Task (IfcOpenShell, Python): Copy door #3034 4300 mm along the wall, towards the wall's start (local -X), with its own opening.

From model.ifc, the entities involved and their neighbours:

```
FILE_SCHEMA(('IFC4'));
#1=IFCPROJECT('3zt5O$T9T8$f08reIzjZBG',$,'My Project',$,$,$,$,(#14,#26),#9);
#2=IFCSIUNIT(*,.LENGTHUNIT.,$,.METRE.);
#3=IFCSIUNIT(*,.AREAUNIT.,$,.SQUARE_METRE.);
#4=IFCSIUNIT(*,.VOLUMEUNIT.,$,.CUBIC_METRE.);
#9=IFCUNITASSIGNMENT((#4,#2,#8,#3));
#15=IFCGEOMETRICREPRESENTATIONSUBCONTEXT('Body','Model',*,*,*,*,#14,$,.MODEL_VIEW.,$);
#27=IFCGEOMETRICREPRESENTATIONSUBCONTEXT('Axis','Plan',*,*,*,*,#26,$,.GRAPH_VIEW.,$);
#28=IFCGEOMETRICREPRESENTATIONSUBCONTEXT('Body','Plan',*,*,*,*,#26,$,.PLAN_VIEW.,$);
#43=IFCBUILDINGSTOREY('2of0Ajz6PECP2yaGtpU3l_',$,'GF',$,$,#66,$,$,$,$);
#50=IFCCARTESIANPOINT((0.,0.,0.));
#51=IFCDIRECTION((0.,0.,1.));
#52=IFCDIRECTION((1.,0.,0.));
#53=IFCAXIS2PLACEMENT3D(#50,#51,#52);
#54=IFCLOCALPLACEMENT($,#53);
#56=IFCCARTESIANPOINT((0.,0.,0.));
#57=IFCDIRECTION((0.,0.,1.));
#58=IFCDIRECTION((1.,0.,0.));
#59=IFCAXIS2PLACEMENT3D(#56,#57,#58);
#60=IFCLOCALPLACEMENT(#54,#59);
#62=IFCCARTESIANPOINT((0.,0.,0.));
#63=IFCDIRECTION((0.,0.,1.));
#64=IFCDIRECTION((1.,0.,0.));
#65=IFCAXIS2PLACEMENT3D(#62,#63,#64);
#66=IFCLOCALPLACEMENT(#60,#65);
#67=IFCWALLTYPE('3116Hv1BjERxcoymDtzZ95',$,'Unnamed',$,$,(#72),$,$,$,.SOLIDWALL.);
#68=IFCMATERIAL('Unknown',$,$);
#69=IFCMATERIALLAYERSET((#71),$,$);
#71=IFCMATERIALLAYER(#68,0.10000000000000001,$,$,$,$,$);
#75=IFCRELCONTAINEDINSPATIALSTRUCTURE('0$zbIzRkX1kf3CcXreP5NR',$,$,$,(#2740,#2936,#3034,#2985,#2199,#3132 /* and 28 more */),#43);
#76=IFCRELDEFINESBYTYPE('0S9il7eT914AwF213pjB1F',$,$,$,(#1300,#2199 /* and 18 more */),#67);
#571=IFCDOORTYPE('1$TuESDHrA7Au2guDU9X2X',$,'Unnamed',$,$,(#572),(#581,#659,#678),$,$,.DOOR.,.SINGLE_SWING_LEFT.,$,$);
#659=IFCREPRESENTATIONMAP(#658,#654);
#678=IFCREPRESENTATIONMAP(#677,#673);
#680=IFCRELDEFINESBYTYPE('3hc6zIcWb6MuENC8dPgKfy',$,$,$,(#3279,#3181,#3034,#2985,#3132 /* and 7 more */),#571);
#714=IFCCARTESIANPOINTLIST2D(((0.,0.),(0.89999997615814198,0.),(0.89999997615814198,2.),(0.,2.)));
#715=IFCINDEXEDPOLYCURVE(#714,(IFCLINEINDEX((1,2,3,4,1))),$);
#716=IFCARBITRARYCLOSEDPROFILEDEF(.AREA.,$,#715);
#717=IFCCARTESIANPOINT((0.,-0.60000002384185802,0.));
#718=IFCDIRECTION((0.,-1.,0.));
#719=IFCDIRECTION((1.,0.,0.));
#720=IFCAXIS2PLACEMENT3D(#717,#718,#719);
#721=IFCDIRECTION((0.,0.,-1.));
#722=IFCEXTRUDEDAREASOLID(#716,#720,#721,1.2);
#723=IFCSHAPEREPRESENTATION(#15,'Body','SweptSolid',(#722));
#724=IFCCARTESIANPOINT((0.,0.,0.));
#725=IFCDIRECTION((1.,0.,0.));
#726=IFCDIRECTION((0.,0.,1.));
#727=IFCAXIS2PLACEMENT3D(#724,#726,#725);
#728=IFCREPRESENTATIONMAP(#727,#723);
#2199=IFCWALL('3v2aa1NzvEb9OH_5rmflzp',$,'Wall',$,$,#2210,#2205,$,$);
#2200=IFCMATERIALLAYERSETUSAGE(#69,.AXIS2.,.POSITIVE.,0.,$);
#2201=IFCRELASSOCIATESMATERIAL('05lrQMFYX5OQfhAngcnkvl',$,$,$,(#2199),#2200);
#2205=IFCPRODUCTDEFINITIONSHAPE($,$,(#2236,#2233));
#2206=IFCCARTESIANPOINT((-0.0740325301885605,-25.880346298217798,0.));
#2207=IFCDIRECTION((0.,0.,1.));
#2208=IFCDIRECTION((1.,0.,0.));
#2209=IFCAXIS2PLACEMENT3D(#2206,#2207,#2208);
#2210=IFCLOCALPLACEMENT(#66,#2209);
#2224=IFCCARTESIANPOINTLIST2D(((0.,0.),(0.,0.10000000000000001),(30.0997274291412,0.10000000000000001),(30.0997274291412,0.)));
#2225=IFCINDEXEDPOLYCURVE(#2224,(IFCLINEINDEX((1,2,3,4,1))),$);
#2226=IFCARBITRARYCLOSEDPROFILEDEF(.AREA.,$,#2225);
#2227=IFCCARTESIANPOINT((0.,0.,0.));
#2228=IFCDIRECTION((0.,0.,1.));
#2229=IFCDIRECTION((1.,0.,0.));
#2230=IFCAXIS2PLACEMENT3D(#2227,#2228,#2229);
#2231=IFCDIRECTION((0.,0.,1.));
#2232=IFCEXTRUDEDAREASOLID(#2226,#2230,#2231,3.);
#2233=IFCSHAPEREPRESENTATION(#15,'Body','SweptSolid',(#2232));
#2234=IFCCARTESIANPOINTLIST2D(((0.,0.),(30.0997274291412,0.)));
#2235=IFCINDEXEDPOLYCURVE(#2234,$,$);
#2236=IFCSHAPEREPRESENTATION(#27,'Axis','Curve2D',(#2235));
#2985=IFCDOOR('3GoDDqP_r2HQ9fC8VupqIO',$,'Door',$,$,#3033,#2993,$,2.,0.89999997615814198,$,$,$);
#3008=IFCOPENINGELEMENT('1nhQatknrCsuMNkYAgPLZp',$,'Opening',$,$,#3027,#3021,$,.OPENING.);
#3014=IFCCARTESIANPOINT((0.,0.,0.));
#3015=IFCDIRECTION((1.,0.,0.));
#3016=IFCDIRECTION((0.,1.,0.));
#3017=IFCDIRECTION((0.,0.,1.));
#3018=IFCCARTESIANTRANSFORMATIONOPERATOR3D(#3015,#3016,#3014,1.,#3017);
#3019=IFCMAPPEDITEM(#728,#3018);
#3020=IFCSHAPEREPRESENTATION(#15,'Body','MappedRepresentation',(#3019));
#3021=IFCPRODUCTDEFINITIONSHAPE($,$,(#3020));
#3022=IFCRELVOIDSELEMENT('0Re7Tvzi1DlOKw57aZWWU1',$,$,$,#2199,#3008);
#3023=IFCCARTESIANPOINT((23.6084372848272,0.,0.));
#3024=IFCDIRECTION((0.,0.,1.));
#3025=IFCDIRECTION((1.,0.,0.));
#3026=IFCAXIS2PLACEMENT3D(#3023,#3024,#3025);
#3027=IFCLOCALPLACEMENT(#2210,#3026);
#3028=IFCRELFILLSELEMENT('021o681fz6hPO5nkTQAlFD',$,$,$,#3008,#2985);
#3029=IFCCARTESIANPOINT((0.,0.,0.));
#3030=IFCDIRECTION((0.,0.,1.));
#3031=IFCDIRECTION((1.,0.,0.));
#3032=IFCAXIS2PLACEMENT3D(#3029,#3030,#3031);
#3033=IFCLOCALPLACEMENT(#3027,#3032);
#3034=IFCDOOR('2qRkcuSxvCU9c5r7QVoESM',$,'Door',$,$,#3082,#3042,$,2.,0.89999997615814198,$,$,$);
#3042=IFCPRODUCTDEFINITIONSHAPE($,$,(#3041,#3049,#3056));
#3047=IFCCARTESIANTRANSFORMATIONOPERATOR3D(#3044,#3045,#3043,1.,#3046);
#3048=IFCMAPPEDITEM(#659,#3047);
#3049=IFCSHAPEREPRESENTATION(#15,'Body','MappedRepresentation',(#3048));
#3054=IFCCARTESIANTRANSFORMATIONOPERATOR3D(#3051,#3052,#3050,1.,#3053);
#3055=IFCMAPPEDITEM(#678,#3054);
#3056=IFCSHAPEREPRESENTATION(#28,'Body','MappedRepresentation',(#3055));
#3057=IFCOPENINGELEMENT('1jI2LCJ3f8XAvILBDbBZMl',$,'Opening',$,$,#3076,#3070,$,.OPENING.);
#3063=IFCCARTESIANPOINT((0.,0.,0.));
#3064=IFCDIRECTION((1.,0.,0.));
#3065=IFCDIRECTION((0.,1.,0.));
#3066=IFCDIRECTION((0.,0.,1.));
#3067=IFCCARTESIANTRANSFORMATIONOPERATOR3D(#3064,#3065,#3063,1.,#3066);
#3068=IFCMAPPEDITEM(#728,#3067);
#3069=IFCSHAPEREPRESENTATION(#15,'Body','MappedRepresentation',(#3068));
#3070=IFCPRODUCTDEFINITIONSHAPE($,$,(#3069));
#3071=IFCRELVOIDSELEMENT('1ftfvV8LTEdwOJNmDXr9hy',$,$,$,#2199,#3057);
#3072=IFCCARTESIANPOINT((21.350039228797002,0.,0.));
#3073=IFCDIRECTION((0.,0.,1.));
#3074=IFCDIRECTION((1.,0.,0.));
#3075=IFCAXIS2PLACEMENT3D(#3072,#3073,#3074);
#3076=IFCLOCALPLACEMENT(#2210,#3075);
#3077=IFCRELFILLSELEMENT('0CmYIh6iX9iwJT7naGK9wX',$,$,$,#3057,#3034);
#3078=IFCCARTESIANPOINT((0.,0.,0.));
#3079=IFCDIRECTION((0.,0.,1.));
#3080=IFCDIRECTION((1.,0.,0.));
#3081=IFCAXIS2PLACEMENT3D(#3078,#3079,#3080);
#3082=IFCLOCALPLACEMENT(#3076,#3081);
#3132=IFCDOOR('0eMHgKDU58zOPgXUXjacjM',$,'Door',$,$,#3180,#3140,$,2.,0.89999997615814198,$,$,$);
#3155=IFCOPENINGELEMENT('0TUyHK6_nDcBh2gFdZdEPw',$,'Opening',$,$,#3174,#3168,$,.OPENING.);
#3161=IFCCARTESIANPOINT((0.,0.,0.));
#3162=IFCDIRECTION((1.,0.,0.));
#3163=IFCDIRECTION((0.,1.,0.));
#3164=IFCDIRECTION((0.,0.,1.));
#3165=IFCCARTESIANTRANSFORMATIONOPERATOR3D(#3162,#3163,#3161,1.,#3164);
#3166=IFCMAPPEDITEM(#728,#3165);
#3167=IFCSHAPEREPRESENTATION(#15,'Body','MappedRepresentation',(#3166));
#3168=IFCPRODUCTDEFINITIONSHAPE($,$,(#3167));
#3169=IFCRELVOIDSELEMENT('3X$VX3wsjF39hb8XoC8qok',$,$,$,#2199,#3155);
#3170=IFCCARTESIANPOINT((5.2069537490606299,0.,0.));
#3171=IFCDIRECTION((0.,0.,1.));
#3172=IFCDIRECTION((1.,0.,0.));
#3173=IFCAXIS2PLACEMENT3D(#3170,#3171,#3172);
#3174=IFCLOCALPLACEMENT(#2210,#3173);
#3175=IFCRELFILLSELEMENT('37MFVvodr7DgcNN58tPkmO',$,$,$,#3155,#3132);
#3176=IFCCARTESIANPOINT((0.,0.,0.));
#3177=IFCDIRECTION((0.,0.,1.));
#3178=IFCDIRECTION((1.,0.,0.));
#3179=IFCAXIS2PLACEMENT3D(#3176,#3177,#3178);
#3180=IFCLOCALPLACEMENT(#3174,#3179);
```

```python
import ifcopenshell
import ifcopenshell.api.feature
import ifcopenshell.api.geometry
import ifcopenshell.api.root
import ifcopenshell.geom
import ifcopenshell.util.element
import ifcopenshell.util.placement
import ifcopenshell.util.shape

model = ifcopenshell.open("model.ifc")
settings = ifcopenshell.geom.settings()


def volume(element):
    """Net volume in cubic metres, openings subtracted."""
    shape = ifcopenshell.geom.create_shape(settings, element)
    return ifcopenshell.util.shape.get_volume(shape.geometry)


door = model.by_guid("2qRkcuSxvCU9c5r7QVoESM")
opening = door.FillsVoids[0].RelatingOpeningElement
wall = opening.VoidsElements[0].RelatingBuildingElement
before = volume(wall)
shift = ifcopenshell.util.placement.get_local_placement(wall.ObjectPlacement)[:3, 0] * -4.3

# copy_class copies the void relationship, type, container and properties, but no geometry.
new_opening = ifcopenshell.api.root.copy_class(model, product=opening)
new_opening.Representation = ifcopenshell.util.element.copy_deep(
    model, opening.Representation, exclude=["IfcGeometricRepresentationContext", "IfcRepresentationMap"]
)
new_door = ifcopenshell.api.root.copy_class(model, product=door)
new_door.Representation = ifcopenshell.util.element.copy_deep(
    model, door.Representation, exclude=["IfcGeometricRepresentationContext", "IfcRepresentationMap"]
)
ifcopenshell.api.feature.add_filling(model, opening=new_opening, element=new_door)

for old, new in ((opening, new_opening), (door, new_door)):
    matrix = ifcopenshell.util.placement.get_local_placement(old.ObjectPlacement)
    matrix[:3, 3] += shift
    ifcopenshell.api.geometry.edit_object_placement(model, product=new, matrix=matrix, is_si=False)

after = volume(wall)

print(f"wall volume {before:.3f} -> {after:.3f} m3")

model.write("model-out.ifc")
```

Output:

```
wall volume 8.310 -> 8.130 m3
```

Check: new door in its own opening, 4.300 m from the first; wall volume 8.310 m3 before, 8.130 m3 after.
